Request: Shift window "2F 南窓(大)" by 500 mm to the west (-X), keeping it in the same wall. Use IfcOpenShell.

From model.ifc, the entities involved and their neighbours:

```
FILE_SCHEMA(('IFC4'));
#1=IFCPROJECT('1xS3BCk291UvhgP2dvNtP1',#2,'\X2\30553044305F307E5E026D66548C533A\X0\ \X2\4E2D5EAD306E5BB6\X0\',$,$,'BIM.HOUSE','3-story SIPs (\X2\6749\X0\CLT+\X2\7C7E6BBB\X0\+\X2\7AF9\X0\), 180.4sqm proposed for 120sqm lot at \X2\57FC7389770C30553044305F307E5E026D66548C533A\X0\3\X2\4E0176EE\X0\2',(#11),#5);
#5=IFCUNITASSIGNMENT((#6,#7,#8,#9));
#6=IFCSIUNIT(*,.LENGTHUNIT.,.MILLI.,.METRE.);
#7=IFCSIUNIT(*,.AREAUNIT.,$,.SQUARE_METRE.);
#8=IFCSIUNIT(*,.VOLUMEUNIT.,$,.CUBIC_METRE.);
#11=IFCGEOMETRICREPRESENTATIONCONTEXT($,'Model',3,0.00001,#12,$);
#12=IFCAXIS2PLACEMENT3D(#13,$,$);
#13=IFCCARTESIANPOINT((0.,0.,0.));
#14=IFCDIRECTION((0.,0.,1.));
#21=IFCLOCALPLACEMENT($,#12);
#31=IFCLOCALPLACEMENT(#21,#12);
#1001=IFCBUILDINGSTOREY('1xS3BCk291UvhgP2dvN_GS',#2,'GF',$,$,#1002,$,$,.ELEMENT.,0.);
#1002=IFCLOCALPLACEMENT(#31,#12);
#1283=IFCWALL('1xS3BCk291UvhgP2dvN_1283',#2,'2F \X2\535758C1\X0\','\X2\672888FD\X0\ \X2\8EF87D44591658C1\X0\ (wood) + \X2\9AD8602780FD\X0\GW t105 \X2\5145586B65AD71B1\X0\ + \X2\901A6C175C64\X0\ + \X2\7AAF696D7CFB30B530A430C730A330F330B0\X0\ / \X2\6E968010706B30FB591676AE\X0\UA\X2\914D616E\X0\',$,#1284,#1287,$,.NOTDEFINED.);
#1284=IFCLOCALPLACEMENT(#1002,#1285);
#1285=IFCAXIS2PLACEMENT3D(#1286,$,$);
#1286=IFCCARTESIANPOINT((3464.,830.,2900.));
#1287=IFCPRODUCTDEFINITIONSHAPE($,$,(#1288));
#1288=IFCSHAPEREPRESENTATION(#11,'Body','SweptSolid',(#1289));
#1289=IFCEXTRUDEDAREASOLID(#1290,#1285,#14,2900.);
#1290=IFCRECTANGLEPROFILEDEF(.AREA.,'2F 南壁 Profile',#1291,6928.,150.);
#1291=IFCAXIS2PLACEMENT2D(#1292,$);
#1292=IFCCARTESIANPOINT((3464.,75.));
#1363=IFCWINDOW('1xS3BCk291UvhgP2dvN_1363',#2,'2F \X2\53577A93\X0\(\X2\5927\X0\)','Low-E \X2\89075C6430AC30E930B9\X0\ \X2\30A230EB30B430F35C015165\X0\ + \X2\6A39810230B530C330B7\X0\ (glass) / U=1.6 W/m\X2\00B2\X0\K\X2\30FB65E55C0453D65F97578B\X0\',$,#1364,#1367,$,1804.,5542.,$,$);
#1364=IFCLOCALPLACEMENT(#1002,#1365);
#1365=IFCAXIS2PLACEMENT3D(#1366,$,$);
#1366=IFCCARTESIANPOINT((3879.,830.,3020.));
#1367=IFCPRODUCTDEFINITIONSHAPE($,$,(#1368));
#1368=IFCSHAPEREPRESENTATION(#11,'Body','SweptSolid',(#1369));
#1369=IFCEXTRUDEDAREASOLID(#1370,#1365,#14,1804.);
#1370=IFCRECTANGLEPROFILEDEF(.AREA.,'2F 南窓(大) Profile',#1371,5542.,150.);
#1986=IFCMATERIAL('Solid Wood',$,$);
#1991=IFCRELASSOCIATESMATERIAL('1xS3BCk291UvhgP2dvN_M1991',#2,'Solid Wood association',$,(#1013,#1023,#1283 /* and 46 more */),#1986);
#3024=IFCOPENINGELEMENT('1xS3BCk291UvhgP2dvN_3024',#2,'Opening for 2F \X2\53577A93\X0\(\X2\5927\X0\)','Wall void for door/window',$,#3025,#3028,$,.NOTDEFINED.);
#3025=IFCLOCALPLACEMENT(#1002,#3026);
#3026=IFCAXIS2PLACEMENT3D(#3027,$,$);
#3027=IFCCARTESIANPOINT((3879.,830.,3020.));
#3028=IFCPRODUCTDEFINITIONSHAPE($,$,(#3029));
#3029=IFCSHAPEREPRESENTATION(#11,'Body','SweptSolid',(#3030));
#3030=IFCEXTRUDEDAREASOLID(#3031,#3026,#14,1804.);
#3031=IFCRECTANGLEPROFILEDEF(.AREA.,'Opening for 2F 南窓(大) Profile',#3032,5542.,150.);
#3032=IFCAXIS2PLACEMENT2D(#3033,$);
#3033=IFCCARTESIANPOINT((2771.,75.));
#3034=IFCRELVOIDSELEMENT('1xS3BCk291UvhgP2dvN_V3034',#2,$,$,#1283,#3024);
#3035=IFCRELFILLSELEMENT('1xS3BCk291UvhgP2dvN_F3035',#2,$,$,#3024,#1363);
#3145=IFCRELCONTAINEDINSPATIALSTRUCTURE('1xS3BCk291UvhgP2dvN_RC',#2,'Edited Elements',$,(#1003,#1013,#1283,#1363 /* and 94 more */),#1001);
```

```python
import ifcopenshell
import ifcopenshell.api.geometry
import ifcopenshell.util.placement
import ifcopenshell.util.unit

model = ifcopenshell.open("model.ifc")
unit_scale = ifcopenshell.util.unit.calculate_unit_scale(model)

window = model.by_id(1363)
opening = window.FillsVoids[0].RelatingOpeningElement
wall = opening.VoidsElements[0].RelatingBuildingElement

wall_matrix = ifcopenshell.util.placement.get_local_placement(wall.ObjectPlacement)
shift = wall_matrix[:3, 0] * -0.5 / unit_scale
before = ifcopenshell.util.placement.get_local_placement(window.ObjectPlacement)[:3, 3].copy()

# The window is not placed relative to its opening, so move both.
for product in (opening, window):
    matrix = ifcopenshell.util.placement.get_local_placement(product.ObjectPlacement)
    matrix[:3, 3] += shift
    ifcopenshell.api.geometry.edit_object_placement(model, product=product, matrix=matrix, is_si=False)

after = ifcopenshell.util.placement.get_local_placement(window.ObjectPlacement)[:3, 3]
print("window moved by", (after - before).round(3) + 0.0)

model.write("model_rev.ifc")
```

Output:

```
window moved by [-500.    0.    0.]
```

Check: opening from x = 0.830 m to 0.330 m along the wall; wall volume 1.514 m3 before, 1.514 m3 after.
